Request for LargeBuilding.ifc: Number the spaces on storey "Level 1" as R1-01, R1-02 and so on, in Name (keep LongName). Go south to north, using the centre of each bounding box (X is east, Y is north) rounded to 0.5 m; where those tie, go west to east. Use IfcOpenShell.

First a look at what the model holds.

```python
import ifcopenshell
import ifcopenshell.util.element
import ifcopenshell.util.placement

model = ifcopenshell.open("LargeBuilding.ifc")
print(model.schema)
storey = next(s for s in model.by_type("IfcBuildingStorey") if s.Name == "Level 1")
spaces = [e for e in ifcopenshell.util.element.get_decomposition(storey) if e.is_a("IfcSpace")]
for e in sorted(spaces, key=lambda e: e.id()):
    origin = ifcopenshell.util.placement.get_local_placement(e.ObjectPlacement)[:3, 3]
    print(e.id(), e.Name, e.LongName, origin.round(2) + 0.0, sep=" | ")
```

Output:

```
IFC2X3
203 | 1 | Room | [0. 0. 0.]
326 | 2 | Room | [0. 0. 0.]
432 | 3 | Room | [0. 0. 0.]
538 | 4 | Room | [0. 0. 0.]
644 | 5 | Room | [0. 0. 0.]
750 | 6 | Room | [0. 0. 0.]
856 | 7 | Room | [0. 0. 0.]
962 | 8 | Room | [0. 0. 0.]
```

```python
import ifcopenshell
import ifcopenshell.geom
import ifcopenshell.util.element
import ifcopenshell.util.shape

model = ifcopenshell.open("LargeBuilding.ifc")
settings = ifcopenshell.geom.settings()
settings.set("use-world-coords", True)


def centre(element):
    shape = ifcopenshell.geom.create_shape(settings, element)
    return ifcopenshell.util.shape.get_bbox_centroid(shape.geometry)


storey = next(s for s in model.by_type("IfcBuildingStorey") if s.Name == "Level 1")
spaces = [e for e in ifcopenshell.util.element.get_decomposition(storey) if e.is_a("IfcSpace")]

# Insertion points can sit at a corner or the storey origin, so sort by the geometry (in metres).
centres = {e: centre(e) for e in spaces}
spaces.sort(key=lambda e: (round(centres[e][1] / 0.5), centres[e][0]))

for i, e in enumerate(spaces, start=1):
    number = f"R1-{i:02d}"
    e.Name = number
    print(e.id(), number)

model.write("LargeBuilding_rev.ifc")
```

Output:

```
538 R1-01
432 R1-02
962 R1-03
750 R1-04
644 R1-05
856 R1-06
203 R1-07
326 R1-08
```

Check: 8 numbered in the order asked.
